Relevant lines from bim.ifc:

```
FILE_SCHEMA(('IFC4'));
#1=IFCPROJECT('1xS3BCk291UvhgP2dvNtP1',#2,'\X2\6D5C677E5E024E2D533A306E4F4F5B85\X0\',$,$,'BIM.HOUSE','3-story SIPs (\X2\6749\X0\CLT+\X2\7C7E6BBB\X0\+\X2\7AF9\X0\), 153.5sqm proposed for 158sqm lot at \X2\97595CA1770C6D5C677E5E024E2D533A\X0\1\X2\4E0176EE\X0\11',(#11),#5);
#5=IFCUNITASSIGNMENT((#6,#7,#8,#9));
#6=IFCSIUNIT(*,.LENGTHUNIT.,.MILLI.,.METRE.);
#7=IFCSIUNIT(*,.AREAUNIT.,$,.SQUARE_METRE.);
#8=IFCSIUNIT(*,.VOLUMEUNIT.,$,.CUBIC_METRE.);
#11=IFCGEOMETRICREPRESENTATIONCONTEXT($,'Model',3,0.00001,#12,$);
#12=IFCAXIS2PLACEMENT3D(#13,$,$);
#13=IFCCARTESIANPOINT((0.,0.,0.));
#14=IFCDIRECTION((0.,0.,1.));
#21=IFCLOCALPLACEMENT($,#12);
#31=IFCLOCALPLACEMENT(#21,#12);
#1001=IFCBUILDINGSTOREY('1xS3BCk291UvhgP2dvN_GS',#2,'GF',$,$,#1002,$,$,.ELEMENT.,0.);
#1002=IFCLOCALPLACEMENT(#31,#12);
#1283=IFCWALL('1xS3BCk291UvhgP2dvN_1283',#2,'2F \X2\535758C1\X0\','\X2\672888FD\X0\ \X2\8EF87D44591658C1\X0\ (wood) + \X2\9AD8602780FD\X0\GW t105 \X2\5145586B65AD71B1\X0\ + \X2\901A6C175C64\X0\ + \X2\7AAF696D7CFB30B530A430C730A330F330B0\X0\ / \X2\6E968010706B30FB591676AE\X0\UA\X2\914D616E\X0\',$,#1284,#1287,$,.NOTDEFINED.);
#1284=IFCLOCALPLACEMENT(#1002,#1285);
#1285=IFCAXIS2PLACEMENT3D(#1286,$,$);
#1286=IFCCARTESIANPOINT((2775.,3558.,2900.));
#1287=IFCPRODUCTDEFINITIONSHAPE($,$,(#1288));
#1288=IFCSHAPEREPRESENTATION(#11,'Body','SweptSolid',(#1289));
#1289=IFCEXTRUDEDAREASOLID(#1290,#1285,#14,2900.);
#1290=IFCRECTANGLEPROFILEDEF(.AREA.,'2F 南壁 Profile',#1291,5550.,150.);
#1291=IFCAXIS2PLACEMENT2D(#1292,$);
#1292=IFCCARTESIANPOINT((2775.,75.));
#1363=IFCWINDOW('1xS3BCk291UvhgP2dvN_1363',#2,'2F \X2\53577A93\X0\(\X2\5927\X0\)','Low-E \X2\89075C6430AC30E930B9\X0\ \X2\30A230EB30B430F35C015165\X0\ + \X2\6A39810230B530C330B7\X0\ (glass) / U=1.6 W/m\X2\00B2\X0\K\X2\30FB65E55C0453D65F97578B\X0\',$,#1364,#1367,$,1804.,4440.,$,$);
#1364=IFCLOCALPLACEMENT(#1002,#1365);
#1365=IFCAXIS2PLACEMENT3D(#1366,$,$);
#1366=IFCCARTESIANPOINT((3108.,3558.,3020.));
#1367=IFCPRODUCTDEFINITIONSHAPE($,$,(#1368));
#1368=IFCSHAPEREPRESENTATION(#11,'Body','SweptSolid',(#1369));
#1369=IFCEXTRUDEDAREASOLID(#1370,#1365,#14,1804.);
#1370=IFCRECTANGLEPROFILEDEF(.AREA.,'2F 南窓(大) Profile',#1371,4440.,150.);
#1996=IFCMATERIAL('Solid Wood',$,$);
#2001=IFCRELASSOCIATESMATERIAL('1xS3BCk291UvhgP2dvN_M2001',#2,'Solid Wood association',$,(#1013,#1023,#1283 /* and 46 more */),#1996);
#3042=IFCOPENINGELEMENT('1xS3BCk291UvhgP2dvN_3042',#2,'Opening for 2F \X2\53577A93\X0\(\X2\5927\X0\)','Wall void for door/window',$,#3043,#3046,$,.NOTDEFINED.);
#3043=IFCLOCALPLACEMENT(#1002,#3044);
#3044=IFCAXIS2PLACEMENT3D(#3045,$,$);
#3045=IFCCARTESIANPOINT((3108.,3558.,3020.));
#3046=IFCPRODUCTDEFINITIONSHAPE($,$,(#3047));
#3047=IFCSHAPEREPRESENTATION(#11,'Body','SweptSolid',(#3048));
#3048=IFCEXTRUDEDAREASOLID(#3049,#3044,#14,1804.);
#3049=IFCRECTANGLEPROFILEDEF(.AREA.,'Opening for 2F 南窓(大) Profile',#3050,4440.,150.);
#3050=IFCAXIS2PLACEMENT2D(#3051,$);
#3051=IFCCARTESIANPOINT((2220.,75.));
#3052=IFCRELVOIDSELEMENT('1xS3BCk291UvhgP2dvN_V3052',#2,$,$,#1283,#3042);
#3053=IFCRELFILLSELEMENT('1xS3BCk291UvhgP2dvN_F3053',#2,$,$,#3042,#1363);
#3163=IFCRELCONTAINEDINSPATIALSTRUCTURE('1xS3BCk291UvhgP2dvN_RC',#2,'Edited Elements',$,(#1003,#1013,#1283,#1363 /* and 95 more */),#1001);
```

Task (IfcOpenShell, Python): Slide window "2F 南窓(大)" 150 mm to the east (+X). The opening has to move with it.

```python
import ifcopenshell
import ifcopenshell.api.geometry
import ifcopenshell.util.placement

model = ifcopenshell.open("bim.ifc")

window = model.by_guid("1xS3BCk291UvhgP2dvN_1363")
opening = window.FillsVoids[0].RelatingOpeningElement
wall = opening.VoidsElements[0].RelatingBuildingElement

wall_matrix = ifcopenshell.util.placement.get_local_placement(wall.ObjectPlacement)
shift = wall_matrix[:3, 0] * 150.0
before = ifcopenshell.util.placement.get_local_placement(window.ObjectPlacement)[:3, 3].copy()

# The window is not placed relative to its opening, so move both.
for product in (opening, window):
    matrix = ifcopenshell.util.placement.get_local_placement(product.ObjectPlacement)
    matrix[:3, 3] += shift
    ifcopenshell.api.geometry.edit_object_placement(model, product=product, matrix=matrix, is_si=False)

after = ifcopenshell.util.placement.get_local_placement(window.ObjectPlacement)[:3, 3]
print("window moved by", (after - before).round(3) + 0.0)

model.write("bim_updated.ifc")
```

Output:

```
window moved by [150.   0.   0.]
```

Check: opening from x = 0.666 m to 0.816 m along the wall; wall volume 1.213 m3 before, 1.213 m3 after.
